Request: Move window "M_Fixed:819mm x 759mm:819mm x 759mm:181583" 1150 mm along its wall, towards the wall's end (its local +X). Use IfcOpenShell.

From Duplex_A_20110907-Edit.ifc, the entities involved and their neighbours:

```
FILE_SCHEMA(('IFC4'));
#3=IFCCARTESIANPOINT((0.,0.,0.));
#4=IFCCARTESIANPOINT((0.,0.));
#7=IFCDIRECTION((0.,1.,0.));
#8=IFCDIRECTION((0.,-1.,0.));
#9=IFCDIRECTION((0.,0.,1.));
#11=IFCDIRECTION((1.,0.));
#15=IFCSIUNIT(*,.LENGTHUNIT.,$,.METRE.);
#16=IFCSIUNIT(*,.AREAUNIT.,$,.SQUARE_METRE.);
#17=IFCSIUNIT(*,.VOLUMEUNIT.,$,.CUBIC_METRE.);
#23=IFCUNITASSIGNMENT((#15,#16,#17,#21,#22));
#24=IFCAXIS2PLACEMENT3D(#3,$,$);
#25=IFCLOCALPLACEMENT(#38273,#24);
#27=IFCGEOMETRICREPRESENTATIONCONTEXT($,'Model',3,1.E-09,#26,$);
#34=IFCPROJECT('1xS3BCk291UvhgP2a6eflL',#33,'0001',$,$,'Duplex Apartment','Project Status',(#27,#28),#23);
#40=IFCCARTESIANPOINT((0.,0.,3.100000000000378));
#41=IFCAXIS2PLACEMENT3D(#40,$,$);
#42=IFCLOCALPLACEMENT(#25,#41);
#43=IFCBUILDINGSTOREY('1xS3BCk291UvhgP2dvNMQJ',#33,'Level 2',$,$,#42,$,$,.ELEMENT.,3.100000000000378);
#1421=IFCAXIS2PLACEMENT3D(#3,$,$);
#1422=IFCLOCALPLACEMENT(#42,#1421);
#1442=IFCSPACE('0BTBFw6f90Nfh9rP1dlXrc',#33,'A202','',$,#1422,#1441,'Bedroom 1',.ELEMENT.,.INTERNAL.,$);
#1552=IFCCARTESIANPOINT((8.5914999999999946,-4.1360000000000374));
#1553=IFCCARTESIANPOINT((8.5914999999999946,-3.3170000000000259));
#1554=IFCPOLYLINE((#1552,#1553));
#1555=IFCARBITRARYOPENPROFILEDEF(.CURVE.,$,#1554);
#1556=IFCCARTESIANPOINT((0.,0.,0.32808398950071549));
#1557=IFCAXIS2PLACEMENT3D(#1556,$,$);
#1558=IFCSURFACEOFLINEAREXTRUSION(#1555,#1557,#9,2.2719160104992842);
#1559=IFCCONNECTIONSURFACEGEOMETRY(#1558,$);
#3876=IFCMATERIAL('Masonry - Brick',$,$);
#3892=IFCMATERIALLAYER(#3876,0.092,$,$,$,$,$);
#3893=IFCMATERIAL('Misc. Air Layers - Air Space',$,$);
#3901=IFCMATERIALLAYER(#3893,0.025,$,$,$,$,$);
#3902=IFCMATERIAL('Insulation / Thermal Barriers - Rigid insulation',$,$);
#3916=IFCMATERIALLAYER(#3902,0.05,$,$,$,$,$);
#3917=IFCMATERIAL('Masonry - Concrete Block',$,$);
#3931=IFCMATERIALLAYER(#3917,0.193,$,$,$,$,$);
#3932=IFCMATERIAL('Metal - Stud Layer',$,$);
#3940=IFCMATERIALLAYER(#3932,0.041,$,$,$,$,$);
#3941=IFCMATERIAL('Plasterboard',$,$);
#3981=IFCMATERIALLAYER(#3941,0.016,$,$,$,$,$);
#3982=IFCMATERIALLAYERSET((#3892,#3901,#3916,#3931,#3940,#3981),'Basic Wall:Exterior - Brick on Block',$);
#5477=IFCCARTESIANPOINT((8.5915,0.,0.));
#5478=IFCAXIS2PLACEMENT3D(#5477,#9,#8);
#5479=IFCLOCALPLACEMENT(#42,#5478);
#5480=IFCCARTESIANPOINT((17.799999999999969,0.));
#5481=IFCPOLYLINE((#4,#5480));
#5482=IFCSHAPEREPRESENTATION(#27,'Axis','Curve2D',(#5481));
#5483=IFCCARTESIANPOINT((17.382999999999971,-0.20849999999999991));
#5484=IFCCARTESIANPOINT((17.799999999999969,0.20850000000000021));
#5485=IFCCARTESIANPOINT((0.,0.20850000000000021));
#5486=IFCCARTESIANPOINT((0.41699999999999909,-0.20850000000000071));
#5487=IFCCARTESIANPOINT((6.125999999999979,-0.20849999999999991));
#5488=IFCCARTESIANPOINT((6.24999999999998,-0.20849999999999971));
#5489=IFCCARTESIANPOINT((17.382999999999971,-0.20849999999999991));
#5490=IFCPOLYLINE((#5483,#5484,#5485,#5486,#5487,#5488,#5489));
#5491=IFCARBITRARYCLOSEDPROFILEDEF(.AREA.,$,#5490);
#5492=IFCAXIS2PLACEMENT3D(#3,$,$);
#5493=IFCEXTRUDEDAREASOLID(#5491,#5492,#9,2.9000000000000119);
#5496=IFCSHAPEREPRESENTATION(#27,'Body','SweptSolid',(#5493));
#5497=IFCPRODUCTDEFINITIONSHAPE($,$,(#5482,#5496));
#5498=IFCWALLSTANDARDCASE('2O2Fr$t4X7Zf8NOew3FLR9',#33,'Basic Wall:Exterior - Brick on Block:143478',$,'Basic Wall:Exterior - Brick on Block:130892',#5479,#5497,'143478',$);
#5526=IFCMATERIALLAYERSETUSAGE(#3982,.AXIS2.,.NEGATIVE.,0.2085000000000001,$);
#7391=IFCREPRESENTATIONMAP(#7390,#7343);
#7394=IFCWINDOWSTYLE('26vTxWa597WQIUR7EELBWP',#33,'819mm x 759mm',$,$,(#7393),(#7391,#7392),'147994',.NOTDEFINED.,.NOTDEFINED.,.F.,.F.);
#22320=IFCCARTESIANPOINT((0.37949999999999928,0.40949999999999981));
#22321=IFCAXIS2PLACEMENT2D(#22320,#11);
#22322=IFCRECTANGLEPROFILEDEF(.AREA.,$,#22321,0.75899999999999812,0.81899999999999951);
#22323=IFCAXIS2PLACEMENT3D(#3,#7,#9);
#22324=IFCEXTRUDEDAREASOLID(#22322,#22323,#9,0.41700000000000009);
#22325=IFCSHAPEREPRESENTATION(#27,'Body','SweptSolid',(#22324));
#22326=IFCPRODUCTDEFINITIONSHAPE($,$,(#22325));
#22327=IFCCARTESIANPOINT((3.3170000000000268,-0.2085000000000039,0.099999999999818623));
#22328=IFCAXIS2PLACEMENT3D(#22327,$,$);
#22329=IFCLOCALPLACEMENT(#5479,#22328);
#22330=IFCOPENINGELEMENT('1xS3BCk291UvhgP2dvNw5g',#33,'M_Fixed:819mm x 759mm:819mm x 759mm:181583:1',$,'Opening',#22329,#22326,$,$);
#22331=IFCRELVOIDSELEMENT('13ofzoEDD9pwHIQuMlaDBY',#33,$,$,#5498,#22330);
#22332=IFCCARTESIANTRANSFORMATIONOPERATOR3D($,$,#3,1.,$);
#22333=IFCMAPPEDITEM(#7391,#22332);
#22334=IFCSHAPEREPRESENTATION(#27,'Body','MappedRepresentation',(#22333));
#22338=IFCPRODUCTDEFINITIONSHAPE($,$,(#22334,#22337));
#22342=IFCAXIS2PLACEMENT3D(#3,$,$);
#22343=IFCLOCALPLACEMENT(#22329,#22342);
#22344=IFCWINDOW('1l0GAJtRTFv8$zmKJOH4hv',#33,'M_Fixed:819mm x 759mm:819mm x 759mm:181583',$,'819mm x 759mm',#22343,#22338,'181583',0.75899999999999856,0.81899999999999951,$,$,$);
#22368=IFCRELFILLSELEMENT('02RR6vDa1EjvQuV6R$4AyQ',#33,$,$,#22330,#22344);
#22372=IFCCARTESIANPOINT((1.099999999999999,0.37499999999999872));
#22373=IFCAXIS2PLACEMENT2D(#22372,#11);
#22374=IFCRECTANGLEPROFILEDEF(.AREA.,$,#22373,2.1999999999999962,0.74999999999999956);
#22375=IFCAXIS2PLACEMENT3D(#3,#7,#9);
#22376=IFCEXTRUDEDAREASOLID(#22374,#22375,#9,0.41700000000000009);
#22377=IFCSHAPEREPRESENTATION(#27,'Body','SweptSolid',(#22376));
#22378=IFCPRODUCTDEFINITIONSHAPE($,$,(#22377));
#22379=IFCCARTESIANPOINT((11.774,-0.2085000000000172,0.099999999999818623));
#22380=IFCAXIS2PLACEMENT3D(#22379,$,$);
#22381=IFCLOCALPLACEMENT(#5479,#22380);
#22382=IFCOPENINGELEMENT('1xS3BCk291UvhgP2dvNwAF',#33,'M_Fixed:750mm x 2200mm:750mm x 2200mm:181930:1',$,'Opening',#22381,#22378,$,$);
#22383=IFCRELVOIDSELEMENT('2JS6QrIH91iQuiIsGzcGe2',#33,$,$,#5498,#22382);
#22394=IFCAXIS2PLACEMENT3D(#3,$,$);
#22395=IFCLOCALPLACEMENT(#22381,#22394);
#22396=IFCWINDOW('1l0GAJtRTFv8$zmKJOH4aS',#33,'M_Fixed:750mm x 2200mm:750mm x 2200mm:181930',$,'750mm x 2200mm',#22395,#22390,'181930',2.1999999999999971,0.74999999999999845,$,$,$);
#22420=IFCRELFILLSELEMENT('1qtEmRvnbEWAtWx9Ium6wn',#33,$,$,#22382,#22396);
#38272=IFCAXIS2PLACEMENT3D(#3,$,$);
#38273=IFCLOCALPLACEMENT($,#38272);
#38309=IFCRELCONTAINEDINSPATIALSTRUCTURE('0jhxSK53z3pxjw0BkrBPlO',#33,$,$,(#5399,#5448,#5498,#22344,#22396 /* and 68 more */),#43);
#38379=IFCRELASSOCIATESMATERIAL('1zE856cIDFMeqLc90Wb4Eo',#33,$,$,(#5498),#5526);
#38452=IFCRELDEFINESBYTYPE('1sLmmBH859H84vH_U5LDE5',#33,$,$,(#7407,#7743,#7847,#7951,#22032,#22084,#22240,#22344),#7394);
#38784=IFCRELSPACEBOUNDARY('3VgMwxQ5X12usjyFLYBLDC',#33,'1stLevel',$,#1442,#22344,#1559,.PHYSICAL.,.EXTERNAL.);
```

```python
import numpy as np
import ifcopenshell
import ifcopenshell.api.geometry
import ifcopenshell.util.placement
import ifcopenshell.util.unit

model = ifcopenshell.open("Duplex_A_20110907-Edit.ifc")
unit_scale = ifcopenshell.util.unit.calculate_unit_scale(model)

window = model.by_guid("1l0GAJtRTFv8$zmKJOH4hv")
opening = window.FillsVoids[0].RelatingOpeningElement
wall = opening.VoidsElements[0].RelatingBuildingElement

wall_matrix = ifcopenshell.util.placement.get_local_placement(wall.ObjectPlacement)
shift = wall_matrix[:3, 0] * 1.15 / unit_scale
before = ifcopenshell.util.placement.get_local_placement(window.ObjectPlacement)[:3, 3].copy()

# The window is placed relative to its opening, so it follows when the opening moves.
matrix = ifcopenshell.util.placement.get_local_placement(opening.ObjectPlacement)
matrix[:3, 3] += shift
ifcopenshell.api.geometry.edit_object_placement(
    model, product=opening, matrix=matrix, is_si=False, should_transform_children=True
)

# Space boundary surfaces are stored in each space's coordinates; move them too.
for rel in window.ProvidesBoundaries:
    if not rel.ConnectionGeometry:
        continue
    surface = rel.ConnectionGeometry.SurfaceOnRelatingElement
    space_matrix = ifcopenshell.util.placement.get_local_placement(rel.RelatingSpace.ObjectPlacement)
    point = np.array(surface.Position.Location.Coordinates) + space_matrix[:3, :3].T @ shift
    surface.Position = model.createIfcAxis2Placement3D(
        model.createIfcCartesianPoint(point.tolist()), surface.Position.Axis, surface.Position.RefDirection
    )

after = ifcopenshell.util.placement.get_local_placement(window.ObjectPlacement)[:3, 3]
print("window moved by", (after - before).round(3) + 0.0)

model.write("Duplex_A_20110907-Edit_updated.ifc")
```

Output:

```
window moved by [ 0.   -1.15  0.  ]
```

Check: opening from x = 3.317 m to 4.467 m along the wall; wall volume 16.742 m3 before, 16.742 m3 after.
